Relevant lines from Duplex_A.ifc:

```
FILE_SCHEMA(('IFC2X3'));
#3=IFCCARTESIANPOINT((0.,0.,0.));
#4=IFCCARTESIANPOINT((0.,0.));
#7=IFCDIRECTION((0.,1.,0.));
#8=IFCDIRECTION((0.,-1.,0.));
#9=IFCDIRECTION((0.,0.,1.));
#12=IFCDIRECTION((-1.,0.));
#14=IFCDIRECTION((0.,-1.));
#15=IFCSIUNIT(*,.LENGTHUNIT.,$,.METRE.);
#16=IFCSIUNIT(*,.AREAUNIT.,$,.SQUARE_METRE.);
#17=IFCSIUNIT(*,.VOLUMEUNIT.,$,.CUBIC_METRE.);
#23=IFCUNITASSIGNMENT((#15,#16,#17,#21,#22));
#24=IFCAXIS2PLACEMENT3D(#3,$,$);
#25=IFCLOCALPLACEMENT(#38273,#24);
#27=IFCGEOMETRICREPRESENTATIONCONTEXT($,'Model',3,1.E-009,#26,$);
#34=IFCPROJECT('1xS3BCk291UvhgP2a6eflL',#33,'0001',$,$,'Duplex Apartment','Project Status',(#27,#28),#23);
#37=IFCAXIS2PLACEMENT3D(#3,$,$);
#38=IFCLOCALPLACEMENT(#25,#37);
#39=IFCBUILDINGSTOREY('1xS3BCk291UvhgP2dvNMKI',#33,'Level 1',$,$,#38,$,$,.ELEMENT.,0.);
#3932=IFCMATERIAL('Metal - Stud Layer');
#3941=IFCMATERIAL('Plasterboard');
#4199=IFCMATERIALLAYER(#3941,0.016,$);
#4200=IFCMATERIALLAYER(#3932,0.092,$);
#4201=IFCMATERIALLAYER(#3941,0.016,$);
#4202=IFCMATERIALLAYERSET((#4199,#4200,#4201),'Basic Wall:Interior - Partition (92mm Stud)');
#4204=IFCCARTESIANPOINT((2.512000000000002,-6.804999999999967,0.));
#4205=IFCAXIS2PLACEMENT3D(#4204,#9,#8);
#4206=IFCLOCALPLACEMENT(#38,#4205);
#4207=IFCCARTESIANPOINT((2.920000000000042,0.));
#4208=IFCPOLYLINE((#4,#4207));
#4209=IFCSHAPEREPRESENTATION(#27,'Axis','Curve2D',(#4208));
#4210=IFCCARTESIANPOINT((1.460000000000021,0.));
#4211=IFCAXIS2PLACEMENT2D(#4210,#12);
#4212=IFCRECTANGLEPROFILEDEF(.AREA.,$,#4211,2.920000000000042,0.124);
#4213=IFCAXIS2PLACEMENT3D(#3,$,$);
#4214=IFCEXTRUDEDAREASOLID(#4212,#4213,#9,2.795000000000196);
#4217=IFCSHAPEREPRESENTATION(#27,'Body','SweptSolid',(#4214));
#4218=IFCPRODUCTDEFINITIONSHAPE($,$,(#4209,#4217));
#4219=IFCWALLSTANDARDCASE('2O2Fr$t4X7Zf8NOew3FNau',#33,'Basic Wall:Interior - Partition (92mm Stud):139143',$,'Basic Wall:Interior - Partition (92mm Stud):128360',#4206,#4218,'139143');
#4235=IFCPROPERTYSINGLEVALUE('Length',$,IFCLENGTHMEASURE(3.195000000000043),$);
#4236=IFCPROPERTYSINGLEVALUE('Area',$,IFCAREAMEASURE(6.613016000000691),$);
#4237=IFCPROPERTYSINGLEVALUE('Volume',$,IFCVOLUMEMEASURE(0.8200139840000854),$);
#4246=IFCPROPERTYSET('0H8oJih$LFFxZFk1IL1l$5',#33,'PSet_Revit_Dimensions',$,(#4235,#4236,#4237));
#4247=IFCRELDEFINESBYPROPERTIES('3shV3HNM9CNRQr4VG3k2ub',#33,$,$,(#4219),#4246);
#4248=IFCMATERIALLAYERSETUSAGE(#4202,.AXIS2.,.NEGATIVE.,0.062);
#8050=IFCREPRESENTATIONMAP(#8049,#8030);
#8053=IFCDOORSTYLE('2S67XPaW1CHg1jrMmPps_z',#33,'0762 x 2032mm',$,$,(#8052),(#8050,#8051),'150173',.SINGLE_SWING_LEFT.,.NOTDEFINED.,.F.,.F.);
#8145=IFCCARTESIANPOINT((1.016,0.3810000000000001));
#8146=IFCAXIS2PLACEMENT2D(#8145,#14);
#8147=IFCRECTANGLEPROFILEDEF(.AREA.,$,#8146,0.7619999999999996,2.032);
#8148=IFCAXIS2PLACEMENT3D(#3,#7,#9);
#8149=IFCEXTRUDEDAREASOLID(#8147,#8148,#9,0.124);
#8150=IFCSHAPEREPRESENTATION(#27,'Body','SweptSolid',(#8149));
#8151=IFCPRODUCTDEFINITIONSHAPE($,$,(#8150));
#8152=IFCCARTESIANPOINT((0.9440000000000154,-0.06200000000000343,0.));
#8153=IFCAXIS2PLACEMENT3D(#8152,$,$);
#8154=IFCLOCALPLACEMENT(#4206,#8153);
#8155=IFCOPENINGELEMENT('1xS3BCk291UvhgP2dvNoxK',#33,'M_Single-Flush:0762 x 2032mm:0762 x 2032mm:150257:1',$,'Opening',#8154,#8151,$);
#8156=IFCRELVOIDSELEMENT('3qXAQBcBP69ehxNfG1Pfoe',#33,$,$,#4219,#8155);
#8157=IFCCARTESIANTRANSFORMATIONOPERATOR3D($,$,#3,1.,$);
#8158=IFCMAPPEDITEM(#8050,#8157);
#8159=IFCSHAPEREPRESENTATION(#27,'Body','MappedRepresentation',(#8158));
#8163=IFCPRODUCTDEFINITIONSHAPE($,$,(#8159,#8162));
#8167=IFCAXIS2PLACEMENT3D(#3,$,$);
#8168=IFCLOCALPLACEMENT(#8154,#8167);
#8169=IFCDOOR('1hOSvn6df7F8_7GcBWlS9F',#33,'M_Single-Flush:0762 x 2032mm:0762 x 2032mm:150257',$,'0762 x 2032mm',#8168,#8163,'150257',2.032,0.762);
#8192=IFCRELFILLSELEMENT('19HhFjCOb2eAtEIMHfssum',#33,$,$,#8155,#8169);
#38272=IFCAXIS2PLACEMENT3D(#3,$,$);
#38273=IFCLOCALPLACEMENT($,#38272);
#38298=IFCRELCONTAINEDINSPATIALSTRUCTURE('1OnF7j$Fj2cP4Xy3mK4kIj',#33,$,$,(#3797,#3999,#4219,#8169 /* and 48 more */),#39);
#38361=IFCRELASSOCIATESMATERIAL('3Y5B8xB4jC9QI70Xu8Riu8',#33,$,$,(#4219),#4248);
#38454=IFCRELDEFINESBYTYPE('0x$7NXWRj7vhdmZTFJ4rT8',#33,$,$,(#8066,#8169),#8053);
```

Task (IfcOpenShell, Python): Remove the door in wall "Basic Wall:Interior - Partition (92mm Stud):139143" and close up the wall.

```python
import ifcopenshell
import ifcopenshell.api.feature
import ifcopenshell.api.pset
import ifcopenshell.api.root
import ifcopenshell.geom
import ifcopenshell.util.element
import ifcopenshell.util.shape
import ifcopenshell.util.unit

model = ifcopenshell.open("Duplex_A.ifc")
area_scale = ifcopenshell.util.unit.calculate_unit_scale(model, "AREAUNIT")
volume_scale = ifcopenshell.util.unit.calculate_unit_scale(model, "VOLUMEUNIT")
settings = ifcopenshell.geom.settings()


def volume(element):
    """Net volume in cubic metres, openings subtracted."""
    shape = ifcopenshell.geom.create_shape(settings, element)
    return ifcopenshell.util.shape.get_volume(shape.geometry)


door = model.by_id(8169)
opening = door.FillsVoids[0].RelatingOpeningElement
wall = opening.VoidsElements[0].RelatingBuildingElement
before = volume(wall)

ifcopenshell.api.root.remove_product(model, product=door)
ifcopenshell.api.feature.remove_feature(model, feature=opening)

after = volume(wall)
thickness = 0.124  # wall thickness in metres

# Update the wall's stored quantities.
pset = model.by_id(ifcopenshell.util.element.get_pset(wall, "PSet_Revit_Dimensions", should_inherit=False)["id"])
ifcopenshell.api.pset.edit_pset(model, pset=pset, properties={
    "Area": model.create_entity("IfcAreaMeasure", after / thickness / area_scale),
    "Volume": model.create_entity("IfcVolumeMeasure", after / volume_scale),
})

print(f"wall volume {before:.3f} -> {after:.3f} m3")

model.write("Duplex_A_v2.ifc")
```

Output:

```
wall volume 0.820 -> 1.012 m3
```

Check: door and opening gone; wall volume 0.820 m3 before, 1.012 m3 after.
